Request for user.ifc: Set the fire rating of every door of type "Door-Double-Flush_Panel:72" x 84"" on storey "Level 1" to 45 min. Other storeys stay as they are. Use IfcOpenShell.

First a look at what the model holds.

```python
import ifcopenshell
import ifcopenshell.util.element

model = ifcopenshell.open("user.ifc")
print(model.schema)
storey = next(s for s in model.by_type("IfcBuildingStorey") if s.Name == "Level 1")
doors = [e for e in ifcopenshell.util.element.get_decomposition(storey) if e.is_a("IfcDoor")]
seen = {}
for e in doors:
    element_type = ifcopenshell.util.element.get_type(e)
    key = (element_type.Name if element_type != e and element_type else None, ifcopenshell.util.element.get_pset(e, "Pset_DoorCommon", "FireRating"))
    seen[key] = seen.get(key, 0) + 1
for (name, value), count in sorted(seen.items(), key=str):
    print(count, "x", name, "|", value)
```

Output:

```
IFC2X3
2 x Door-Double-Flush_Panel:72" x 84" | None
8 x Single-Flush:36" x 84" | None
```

```python
import ifcopenshell
import ifcopenshell.api.pset
import ifcopenshell.util.element

model = ifcopenshell.open("user.ifc")

storey = next(s for s in model.by_type("IfcBuildingStorey") if s.Name == "Level 1")
doors = [e for e in ifcopenshell.util.element.get_decomposition(storey) if e.is_a("IfcDoor")]

count = 0
for e in doors:
    element_type = ifcopenshell.util.element.get_type(e)
    if element_type in (None, e) or element_type.Name != 'Door-Double-Flush_Panel:72" x 84"':
        continue
    # add_pset returns the element's existing set when there is one.
    pset = ifcopenshell.api.pset.add_pset(model, product=e, name="Pset_DoorCommon")
    ifcopenshell.api.pset.edit_pset(model, pset=pset, properties={"FireRating": "45 min"})
    count += 1

print(count, "doors updated")

model.write("user_v2.ifc")
```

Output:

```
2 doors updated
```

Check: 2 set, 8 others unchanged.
